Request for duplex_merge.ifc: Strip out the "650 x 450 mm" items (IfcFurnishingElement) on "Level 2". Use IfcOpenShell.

First a look at what the model holds.

```python
import ifcopenshell
import ifcopenshell.util.element

model = ifcopenshell.open("duplex_merge.ifc")
print(model.schema)
storey = next(s for s in model.by_type("IfcBuildingStorey") if s.Name == "Level 2")
furniture = [e for e in ifcopenshell.util.element.get_decomposition(storey) if e.is_a("IfcFurnishingElement")]
seen = {}
for e in furniture:
    element_type = ifcopenshell.util.element.get_type(e)
    name = element_type.Name if element_type not in (None, e) else None
    seen[name] = seen.get(name, 0) + 1
for name, count in sorted(seen.items(), key=str):
    print(count, "x", name)
```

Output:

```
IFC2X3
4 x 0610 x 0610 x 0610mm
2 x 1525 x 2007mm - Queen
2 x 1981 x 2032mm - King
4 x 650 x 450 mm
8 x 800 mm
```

```python
import ifcopenshell
import ifcopenshell.api.root
import ifcopenshell.util.element

model = ifcopenshell.open("duplex_merge.ifc")

storey = next(s for s in model.by_type("IfcBuildingStorey") if s.Name == "Level 2")
furniture = [e for e in ifcopenshell.util.element.get_decomposition(storey) if e.is_a("IfcFurnishingElement")]
targets = [e for e in furniture if (t := ifcopenshell.util.element.get_type(e)) not in (None, e) and t.Name == "650 x 450 mm"]

for e in targets:
    ifcopenshell.api.root.remove_product(model, product=e)
print(len(targets), "removed")

model.write("duplex_merge-out.ifc")
```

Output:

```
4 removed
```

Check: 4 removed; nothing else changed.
